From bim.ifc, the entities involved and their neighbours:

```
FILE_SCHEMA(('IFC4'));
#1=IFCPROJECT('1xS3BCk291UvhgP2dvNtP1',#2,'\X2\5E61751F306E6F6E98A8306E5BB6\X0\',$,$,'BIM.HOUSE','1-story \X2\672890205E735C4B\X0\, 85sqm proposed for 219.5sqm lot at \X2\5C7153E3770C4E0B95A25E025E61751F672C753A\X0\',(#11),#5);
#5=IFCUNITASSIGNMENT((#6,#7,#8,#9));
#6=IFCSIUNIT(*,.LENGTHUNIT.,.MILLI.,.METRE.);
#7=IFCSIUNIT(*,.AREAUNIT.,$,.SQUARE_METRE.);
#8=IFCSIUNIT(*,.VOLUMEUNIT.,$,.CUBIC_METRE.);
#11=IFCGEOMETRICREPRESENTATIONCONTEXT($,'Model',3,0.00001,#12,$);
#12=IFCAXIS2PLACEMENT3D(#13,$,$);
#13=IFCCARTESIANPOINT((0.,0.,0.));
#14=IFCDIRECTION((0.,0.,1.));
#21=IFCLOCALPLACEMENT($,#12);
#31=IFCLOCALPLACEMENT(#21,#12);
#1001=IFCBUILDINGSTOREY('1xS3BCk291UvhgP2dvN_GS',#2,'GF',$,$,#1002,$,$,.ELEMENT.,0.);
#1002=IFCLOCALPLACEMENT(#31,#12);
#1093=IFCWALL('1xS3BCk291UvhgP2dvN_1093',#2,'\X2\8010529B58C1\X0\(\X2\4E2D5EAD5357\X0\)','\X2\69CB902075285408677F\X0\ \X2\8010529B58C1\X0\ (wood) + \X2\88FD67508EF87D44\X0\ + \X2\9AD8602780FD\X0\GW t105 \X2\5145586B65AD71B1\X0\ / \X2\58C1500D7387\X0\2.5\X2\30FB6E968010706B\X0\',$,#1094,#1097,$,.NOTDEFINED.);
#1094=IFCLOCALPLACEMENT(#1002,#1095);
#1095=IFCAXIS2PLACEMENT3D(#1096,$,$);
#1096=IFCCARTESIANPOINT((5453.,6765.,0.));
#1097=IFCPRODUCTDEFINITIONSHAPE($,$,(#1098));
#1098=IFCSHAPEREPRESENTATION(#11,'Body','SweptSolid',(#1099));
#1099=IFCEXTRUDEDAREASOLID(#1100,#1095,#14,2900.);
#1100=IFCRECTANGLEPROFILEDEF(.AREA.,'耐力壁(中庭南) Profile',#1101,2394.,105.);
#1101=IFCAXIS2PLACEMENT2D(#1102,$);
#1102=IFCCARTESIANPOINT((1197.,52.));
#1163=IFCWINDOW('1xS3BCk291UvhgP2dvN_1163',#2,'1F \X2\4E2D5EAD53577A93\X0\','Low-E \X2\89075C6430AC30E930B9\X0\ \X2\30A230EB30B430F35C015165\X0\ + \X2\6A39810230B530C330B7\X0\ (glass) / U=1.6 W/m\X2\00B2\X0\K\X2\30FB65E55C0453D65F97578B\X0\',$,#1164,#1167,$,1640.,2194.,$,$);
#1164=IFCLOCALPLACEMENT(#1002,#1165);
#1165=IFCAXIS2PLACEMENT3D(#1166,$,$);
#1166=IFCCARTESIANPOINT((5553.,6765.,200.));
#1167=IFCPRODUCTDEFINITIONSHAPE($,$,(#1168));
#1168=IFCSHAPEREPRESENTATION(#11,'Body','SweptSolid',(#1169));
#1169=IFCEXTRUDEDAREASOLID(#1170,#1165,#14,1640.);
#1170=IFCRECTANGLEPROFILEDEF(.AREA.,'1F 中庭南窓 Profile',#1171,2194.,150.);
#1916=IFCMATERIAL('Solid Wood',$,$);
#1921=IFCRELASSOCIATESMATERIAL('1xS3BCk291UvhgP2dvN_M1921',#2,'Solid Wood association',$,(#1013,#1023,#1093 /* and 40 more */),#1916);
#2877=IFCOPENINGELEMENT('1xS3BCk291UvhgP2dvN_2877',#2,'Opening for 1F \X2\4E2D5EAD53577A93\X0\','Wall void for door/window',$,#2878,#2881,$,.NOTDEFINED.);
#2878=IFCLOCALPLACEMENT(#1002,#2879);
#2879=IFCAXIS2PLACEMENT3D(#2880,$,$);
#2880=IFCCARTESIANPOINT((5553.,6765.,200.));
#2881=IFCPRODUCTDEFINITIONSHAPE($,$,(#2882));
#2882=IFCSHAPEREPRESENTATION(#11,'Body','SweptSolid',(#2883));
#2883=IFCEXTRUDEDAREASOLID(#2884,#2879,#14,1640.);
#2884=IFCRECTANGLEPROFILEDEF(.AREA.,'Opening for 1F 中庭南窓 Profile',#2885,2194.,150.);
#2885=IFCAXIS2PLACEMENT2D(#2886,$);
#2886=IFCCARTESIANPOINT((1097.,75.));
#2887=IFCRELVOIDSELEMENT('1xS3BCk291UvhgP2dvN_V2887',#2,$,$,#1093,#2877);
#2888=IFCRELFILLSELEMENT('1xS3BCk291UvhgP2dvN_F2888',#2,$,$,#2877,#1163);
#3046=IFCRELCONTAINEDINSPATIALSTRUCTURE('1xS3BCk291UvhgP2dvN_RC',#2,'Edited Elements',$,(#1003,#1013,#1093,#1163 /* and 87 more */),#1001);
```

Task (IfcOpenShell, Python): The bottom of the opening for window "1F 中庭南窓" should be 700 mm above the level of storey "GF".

```python
import numpy as np
import ifcopenshell
import ifcopenshell.api.geometry
import ifcopenshell.geom
import ifcopenshell.util.element
import ifcopenshell.util.placement
import ifcopenshell.util.shape
import ifcopenshell.util.unit

model = ifcopenshell.open("bim.ifc")
unit_scale = ifcopenshell.util.unit.calculate_unit_scale(model)

window = model.by_guid("1xS3BCk291UvhgP2dvN_1163")
opening = window.FillsVoids[0].RelatingOpeningElement
storey = ifcopenshell.util.element.get_container(window, ifc_class="IfcBuildingStorey")
level = ifcopenshell.util.placement.get_local_placement(storey.ObjectPlacement)[2, 3]

# The opening's origin need not be at the sill, so measure its lowest point.
shape = ifcopenshell.geom.create_shape(ifcopenshell.geom.settings(), opening)
bottom = ifcopenshell.util.shape.get_shape_bottom_elevation(shape, shape.geometry) / unit_scale
dz = level + 700.0 - bottom

shift = np.array([0.0, 0.0, dz])
# The window is not placed relative to its opening, so move both.
for product in (opening, window):
    matrix = ifcopenshell.util.placement.get_local_placement(product.ObjectPlacement)
    matrix[:3, 3] += shift
    ifcopenshell.api.geometry.edit_object_placement(model, product=product, matrix=matrix, is_si=False)

print(f"moved by {dz * unit_scale:+.3f} m")

model.write("bim_rev.ifc")
```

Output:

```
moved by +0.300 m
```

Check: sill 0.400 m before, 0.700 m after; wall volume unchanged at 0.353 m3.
